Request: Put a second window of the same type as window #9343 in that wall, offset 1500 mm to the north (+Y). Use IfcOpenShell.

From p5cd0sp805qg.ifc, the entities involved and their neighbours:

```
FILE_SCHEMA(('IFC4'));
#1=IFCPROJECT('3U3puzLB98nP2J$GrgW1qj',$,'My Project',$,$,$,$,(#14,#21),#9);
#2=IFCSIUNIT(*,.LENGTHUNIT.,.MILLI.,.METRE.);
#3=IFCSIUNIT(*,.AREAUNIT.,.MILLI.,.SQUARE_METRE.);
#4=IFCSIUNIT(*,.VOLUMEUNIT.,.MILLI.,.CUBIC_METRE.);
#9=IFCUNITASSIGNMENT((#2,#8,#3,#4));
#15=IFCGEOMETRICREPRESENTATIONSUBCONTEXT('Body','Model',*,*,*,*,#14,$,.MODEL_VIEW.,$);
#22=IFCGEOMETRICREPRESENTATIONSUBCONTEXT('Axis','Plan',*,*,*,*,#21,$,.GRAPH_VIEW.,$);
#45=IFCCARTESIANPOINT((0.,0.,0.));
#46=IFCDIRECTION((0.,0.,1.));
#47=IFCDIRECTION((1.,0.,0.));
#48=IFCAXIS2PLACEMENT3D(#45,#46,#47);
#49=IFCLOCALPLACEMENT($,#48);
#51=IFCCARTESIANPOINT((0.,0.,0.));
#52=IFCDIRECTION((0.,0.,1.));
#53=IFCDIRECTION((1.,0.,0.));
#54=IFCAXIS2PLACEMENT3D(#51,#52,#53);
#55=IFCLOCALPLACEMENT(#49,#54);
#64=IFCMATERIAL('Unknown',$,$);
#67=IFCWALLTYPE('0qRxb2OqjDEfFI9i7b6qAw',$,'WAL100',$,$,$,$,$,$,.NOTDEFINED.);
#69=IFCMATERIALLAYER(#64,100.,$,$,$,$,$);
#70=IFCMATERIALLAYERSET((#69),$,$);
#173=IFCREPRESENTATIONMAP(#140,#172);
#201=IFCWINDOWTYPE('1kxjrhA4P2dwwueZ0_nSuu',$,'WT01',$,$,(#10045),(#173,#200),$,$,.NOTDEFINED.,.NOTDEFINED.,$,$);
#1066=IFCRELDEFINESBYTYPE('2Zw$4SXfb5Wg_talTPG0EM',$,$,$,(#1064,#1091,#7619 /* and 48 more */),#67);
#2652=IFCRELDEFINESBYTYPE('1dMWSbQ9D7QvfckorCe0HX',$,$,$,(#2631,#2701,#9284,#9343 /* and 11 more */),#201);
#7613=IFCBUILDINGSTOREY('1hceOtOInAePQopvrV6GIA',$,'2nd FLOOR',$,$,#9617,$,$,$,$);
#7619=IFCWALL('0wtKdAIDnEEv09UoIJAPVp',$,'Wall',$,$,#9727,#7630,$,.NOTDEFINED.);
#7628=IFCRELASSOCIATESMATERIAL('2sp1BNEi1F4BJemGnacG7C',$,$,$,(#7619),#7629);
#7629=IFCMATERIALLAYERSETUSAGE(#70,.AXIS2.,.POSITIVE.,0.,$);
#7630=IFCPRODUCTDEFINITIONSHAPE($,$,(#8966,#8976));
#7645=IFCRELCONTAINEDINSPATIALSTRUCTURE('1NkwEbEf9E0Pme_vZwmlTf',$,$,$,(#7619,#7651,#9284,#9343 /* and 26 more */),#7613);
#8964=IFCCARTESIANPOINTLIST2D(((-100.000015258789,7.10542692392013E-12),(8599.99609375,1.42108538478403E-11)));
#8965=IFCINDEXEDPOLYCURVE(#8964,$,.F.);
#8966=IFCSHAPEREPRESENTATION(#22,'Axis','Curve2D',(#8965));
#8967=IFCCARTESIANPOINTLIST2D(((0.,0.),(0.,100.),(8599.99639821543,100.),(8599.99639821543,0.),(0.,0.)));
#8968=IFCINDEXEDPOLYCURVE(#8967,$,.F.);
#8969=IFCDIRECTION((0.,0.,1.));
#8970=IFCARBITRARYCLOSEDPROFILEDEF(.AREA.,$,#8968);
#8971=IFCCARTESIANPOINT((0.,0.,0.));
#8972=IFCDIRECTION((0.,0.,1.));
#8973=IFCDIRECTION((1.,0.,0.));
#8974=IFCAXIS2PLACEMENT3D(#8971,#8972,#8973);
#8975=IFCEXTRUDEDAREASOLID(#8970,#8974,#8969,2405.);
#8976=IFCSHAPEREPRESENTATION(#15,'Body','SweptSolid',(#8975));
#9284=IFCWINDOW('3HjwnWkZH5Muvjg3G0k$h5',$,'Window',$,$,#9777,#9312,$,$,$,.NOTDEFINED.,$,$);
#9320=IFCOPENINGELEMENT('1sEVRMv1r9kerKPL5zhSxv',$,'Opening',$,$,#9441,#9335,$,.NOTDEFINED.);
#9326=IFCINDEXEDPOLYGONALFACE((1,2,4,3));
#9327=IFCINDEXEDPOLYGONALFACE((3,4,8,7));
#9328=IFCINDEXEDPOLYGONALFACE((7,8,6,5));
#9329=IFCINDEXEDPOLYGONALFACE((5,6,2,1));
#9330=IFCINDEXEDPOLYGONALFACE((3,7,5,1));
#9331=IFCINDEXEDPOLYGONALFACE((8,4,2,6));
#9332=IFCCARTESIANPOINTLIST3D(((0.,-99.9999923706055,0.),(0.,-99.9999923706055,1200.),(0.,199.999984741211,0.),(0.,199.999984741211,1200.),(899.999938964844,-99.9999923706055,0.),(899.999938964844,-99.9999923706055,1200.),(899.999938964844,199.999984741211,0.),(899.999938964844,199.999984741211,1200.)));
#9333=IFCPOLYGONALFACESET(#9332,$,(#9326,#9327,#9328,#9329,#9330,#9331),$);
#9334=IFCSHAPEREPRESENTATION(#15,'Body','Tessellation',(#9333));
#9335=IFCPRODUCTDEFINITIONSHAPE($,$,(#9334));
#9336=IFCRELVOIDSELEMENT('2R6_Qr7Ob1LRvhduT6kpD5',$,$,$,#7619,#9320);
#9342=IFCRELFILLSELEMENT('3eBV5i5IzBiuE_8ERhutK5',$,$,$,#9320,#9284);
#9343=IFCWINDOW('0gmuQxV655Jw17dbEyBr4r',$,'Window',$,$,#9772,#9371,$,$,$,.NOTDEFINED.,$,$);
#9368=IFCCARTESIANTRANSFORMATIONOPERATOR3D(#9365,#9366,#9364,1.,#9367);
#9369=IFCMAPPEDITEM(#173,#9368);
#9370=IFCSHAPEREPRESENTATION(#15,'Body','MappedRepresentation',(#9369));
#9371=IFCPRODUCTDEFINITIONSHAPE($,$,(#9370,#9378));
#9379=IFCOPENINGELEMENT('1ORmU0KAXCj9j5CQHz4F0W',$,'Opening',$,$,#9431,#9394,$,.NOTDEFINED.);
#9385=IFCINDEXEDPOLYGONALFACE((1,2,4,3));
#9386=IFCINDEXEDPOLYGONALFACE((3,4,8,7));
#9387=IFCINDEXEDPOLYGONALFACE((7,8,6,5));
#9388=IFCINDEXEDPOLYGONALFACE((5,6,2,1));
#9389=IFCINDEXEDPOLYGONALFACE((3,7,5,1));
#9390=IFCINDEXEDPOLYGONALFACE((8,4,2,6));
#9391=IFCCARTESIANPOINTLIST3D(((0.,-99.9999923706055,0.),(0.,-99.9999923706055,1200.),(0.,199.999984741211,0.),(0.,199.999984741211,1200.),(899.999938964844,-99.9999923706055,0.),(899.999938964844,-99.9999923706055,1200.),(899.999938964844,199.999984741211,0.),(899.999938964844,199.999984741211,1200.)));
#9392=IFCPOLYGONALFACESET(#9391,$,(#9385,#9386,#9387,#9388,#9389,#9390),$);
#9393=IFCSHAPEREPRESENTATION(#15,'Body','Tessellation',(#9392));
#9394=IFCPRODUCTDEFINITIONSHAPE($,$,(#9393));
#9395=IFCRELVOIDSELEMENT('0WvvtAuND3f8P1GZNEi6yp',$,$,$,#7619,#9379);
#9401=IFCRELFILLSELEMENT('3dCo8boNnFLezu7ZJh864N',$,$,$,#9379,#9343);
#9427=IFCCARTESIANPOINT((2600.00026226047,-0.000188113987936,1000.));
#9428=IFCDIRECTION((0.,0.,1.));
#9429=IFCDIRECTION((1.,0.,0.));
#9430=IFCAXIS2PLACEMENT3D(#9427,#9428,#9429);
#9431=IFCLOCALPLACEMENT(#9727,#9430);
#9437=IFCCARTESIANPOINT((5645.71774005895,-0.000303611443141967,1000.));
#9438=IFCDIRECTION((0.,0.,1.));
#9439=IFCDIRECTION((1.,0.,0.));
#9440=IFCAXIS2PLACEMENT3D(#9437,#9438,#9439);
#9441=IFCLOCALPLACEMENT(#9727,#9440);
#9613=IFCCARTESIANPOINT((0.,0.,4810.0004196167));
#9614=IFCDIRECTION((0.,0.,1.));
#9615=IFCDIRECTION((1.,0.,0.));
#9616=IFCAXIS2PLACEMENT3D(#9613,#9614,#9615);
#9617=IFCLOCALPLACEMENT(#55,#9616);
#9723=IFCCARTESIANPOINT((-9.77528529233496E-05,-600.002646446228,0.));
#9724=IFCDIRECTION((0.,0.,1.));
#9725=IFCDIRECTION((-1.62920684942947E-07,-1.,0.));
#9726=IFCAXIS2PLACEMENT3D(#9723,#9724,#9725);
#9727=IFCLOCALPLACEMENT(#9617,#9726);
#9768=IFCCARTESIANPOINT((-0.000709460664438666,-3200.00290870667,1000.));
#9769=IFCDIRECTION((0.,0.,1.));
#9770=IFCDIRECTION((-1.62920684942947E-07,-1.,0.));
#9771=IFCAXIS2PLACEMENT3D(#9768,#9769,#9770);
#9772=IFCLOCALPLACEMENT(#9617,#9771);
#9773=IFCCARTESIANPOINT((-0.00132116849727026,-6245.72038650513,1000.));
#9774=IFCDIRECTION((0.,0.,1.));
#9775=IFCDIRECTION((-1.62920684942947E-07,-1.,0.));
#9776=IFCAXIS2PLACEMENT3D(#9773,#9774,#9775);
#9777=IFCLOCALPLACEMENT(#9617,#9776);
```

```python
import ifcopenshell
import ifcopenshell.api.feature
import ifcopenshell.api.geometry
import ifcopenshell.api.root
import ifcopenshell.geom
import ifcopenshell.util.element
import ifcopenshell.util.placement
import ifcopenshell.util.shape
import ifcopenshell.util.unit

model = ifcopenshell.open("p5cd0sp805qg.ifc")
unit_scale = ifcopenshell.util.unit.calculate_unit_scale(model)
settings = ifcopenshell.geom.settings()


def volume(element):
    """Net volume in cubic metres, openings subtracted."""
    shape = ifcopenshell.geom.create_shape(settings, element)
    return ifcopenshell.util.shape.get_volume(shape.geometry)


window = model.by_id(9343)
opening = window.FillsVoids[0].RelatingOpeningElement
wall = opening.VoidsElements[0].RelatingBuildingElement
before = volume(wall)
shift = ifcopenshell.util.placement.get_local_placement(wall.ObjectPlacement)[:3, 0] * -1.5 / unit_scale

# copy_class copies the void relationship, type, container and properties, but no geometry.
new_opening = ifcopenshell.api.root.copy_class(model, product=opening)
new_opening.Representation = ifcopenshell.util.element.copy_deep(
    model, opening.Representation, exclude=["IfcGeometricRepresentationContext", "IfcRepresentationMap"]
)
new_window = ifcopenshell.api.root.copy_class(model, product=window)
new_window.Representation = ifcopenshell.util.element.copy_deep(
    model, window.Representation, exclude=["IfcGeometricRepresentationContext", "IfcRepresentationMap"]
)
ifcopenshell.api.feature.add_filling(model, opening=new_opening, element=new_window)

for old, new in ((opening, new_opening), (window, new_window)):
    matrix = ifcopenshell.util.placement.get_local_placement(old.ObjectPlacement)
    matrix[:3, 3] += shift
    ifcopenshell.api.geometry.edit_object_placement(model, product=new, matrix=matrix, is_si=False)

after = volume(wall)

print(f"wall volume {before:.3f} -> {after:.3f} m3")

model.write("p5cd0sp805qg_edited.ifc")
```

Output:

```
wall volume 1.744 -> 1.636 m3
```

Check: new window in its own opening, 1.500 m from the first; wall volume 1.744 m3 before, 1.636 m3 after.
